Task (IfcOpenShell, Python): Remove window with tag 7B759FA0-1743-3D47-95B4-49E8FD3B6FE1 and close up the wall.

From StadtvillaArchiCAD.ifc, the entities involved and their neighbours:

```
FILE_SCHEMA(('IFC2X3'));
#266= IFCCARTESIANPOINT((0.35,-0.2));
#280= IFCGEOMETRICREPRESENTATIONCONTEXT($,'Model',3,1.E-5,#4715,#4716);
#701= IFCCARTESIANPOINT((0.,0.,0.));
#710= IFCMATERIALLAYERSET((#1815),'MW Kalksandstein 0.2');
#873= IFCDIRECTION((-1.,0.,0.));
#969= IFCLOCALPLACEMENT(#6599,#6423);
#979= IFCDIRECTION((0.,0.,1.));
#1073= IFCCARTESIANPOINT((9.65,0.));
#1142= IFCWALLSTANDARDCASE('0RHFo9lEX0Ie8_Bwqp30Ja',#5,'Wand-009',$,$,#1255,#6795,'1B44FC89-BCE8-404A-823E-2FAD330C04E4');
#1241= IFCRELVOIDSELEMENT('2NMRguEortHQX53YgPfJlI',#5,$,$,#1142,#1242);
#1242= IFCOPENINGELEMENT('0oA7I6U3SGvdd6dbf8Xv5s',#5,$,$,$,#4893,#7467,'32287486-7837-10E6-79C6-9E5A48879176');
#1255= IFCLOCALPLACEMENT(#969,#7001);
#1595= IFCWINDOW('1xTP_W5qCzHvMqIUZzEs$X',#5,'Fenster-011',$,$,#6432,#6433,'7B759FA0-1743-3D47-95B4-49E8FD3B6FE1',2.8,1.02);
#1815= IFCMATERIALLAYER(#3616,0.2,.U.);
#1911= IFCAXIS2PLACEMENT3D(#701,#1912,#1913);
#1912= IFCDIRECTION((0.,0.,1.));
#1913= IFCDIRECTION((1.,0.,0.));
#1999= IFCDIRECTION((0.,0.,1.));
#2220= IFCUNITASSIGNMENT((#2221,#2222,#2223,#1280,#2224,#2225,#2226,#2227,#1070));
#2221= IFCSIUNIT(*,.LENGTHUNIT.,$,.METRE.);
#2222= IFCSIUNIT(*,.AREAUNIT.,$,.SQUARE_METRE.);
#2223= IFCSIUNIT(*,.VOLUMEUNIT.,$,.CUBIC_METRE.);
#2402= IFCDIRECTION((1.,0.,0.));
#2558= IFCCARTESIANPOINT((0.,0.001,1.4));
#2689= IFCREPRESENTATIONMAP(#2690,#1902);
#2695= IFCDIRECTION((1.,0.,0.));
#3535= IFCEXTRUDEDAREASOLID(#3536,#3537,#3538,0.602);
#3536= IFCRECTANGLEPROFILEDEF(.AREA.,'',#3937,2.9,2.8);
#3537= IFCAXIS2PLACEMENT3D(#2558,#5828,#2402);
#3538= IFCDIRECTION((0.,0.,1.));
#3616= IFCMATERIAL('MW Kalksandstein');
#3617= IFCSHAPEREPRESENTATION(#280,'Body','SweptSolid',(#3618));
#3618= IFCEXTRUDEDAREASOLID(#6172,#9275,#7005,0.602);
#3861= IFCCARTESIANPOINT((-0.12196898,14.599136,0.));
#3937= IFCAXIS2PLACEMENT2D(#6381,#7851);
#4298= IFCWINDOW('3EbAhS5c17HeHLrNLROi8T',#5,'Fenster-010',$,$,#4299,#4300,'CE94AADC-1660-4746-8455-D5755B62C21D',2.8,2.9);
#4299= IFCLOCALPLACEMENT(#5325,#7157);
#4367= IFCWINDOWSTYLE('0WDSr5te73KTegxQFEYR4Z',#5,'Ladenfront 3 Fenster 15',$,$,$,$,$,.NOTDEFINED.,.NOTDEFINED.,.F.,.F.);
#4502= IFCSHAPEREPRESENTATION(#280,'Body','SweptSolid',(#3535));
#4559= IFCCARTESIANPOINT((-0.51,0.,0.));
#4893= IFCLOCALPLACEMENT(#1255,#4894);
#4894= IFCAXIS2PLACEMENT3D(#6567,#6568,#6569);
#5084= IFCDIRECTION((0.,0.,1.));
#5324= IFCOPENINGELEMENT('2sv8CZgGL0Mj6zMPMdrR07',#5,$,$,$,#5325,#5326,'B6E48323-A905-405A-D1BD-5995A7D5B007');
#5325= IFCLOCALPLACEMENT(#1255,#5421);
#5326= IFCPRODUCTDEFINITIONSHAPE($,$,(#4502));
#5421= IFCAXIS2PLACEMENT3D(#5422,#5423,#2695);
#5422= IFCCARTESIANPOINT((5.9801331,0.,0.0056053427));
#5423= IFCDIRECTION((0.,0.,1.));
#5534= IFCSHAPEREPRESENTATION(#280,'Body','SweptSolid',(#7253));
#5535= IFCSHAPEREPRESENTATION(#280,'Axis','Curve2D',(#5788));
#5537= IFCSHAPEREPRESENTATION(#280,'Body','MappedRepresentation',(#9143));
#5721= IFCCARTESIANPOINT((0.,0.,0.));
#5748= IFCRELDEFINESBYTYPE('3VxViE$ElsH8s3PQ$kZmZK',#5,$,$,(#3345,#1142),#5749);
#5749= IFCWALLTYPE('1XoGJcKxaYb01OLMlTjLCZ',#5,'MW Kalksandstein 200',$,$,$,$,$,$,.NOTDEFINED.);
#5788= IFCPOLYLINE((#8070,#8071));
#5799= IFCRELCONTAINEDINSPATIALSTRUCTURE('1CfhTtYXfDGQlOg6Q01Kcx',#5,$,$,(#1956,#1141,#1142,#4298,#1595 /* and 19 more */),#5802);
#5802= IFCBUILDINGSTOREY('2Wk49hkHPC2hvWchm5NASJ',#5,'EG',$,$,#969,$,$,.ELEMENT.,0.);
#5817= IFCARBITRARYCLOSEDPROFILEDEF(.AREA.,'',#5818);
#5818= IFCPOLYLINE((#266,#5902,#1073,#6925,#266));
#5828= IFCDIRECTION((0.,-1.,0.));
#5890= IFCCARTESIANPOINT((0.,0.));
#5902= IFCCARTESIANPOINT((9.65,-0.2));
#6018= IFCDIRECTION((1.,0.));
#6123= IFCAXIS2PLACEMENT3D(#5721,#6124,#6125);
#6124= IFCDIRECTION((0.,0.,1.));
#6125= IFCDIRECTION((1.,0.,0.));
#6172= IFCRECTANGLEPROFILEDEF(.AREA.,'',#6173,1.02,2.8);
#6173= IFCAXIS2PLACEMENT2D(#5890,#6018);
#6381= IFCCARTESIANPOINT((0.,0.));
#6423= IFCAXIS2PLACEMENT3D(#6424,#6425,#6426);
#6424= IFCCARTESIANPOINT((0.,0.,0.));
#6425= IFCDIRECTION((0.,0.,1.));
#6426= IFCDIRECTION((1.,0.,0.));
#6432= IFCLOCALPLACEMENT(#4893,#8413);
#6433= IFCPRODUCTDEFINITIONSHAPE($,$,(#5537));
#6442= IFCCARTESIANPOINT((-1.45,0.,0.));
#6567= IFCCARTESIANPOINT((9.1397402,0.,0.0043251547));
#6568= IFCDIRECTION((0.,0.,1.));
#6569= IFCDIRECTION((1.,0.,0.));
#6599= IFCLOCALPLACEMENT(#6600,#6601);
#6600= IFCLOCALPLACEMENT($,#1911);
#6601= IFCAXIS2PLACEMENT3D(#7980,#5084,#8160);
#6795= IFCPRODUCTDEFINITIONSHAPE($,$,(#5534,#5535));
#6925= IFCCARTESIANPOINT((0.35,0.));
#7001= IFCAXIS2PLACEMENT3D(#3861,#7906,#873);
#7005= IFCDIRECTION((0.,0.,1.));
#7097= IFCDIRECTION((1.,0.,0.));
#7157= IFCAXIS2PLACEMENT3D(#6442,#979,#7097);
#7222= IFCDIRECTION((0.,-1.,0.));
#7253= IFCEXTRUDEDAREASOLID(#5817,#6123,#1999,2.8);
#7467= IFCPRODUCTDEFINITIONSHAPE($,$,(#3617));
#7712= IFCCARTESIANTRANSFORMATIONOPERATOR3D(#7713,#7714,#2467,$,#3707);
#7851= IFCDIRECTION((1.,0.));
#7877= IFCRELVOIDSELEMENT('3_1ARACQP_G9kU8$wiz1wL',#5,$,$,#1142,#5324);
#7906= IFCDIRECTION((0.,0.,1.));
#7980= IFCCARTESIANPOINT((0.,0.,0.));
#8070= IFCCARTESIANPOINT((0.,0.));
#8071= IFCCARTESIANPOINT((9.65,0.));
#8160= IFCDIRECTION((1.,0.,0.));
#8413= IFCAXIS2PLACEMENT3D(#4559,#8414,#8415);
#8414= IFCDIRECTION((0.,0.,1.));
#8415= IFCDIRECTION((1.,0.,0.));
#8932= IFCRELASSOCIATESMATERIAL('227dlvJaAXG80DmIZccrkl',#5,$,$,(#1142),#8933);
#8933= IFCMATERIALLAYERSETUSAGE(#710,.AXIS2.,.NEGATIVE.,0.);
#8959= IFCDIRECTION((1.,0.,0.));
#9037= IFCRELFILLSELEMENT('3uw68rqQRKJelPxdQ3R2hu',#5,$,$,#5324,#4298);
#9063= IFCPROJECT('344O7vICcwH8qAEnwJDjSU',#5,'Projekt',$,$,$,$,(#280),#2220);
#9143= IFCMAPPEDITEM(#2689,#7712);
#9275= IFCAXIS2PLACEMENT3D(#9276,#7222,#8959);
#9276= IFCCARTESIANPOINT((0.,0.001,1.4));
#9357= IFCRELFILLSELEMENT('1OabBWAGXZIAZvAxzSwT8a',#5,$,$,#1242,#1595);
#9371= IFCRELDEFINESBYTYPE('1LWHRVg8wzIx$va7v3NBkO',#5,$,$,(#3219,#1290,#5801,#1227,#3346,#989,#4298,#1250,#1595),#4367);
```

```python
import ifcopenshell
import ifcopenshell.api.feature
import ifcopenshell.api.root
import ifcopenshell.geom
import ifcopenshell.util.shape

model = ifcopenshell.open("StadtvillaArchiCAD.ifc")
settings = ifcopenshell.geom.settings()


def volume(element):
    """Net volume in cubic metres, openings subtracted."""
    shape = ifcopenshell.geom.create_shape(settings, element)
    return ifcopenshell.util.shape.get_volume(shape.geometry)


window = model.by_guid("1xTP_W5qCzHvMqIUZzEs$X")
opening = window.FillsVoids[0].RelatingOpeningElement
wall = opening.VoidsElements[0].RelatingBuildingElement
before = volume(wall)

ifcopenshell.api.root.remove_product(model, product=window)
ifcopenshell.api.feature.remove_feature(model, feature=opening)

after = volume(wall)

print(f"wall volume {before:.3f} -> {after:.3f} m3")

model.write("StadtvillaArchiCAD_edited.ifc")
```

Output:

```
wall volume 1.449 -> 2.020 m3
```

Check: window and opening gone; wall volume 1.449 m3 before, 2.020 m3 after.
